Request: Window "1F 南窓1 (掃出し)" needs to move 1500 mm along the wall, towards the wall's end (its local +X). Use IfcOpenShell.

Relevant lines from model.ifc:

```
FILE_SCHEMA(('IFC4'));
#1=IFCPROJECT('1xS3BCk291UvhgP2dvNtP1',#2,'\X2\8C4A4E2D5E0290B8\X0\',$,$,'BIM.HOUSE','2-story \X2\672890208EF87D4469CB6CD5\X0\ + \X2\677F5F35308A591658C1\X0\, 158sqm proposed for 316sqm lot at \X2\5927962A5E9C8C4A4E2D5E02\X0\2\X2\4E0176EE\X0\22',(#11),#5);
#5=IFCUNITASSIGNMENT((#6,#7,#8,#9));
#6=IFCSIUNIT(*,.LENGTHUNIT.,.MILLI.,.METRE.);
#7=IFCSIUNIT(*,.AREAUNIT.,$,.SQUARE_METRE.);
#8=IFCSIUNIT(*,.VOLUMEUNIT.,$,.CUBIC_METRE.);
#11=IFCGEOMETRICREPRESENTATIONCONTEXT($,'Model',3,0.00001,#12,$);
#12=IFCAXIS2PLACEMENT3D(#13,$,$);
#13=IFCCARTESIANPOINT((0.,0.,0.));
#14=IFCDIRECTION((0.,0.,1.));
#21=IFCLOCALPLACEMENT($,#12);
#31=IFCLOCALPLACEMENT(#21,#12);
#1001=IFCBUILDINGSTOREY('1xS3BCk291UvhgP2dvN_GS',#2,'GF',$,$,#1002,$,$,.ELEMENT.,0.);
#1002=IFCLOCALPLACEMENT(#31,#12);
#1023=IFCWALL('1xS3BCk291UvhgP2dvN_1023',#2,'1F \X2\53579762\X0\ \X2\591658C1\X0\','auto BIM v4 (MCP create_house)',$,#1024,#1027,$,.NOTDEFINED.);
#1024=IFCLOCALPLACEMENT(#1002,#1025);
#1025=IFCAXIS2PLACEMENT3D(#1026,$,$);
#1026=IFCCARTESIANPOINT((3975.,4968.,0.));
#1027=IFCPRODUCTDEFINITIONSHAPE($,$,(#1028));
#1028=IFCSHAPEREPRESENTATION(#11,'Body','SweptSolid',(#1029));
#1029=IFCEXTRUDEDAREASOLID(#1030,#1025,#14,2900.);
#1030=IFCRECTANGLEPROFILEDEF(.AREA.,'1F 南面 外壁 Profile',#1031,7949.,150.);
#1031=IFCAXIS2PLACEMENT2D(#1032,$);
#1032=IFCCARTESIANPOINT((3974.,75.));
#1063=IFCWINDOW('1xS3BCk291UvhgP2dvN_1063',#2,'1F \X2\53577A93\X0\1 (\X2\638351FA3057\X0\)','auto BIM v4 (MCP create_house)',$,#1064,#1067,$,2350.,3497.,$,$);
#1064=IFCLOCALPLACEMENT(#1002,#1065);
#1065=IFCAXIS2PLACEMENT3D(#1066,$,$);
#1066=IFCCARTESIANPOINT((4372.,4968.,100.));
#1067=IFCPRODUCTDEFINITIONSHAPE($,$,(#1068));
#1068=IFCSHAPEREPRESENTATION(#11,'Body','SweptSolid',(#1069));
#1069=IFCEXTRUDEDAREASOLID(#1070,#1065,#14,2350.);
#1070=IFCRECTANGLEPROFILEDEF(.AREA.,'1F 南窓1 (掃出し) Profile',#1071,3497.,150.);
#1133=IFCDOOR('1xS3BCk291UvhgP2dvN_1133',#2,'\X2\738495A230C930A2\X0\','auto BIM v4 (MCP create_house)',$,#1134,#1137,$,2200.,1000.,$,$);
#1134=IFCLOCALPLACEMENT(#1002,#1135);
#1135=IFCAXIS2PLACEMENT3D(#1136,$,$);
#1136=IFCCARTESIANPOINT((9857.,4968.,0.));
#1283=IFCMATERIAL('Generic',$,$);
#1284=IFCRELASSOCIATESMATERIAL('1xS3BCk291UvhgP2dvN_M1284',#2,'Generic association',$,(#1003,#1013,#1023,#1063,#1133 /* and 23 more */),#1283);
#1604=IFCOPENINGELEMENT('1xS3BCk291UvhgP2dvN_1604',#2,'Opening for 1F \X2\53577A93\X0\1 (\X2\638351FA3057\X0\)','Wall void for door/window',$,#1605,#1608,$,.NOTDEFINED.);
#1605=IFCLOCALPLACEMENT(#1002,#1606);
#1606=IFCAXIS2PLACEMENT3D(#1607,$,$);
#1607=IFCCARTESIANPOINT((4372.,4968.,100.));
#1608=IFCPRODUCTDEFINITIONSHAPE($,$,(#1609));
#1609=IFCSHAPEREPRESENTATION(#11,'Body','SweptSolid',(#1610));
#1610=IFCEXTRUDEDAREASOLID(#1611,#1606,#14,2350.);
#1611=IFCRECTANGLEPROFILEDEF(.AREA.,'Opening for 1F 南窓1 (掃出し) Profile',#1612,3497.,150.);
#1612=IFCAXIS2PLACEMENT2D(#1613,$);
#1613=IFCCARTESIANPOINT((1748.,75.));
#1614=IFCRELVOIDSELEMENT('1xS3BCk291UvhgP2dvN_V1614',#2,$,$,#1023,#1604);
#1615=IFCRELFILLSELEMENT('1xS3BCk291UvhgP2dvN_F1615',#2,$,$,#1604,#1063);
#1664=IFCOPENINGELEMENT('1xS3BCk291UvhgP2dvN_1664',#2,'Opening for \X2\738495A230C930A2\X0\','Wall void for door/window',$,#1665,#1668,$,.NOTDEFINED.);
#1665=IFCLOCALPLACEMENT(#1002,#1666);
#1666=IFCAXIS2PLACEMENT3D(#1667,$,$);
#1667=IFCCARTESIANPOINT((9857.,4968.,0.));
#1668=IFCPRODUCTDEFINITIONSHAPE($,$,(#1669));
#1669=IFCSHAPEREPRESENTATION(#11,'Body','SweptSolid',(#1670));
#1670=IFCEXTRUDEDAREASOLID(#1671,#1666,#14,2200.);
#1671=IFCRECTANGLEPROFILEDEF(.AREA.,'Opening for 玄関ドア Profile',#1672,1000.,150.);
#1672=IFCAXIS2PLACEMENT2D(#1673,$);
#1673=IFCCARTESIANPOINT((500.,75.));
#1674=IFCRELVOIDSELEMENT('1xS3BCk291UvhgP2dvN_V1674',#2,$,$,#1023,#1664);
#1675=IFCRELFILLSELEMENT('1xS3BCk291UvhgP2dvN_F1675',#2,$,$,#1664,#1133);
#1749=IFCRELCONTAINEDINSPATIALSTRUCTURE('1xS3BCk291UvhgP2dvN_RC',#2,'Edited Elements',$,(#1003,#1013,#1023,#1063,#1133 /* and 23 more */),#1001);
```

```python
import ifcopenshell
import ifcopenshell.api.geometry
import ifcopenshell.util.placement

model = ifcopenshell.open("model.ifc")

window = model.by_id(1063)
opening = window.FillsVoids[0].RelatingOpeningElement
wall = opening.VoidsElements[0].RelatingBuildingElement

wall_matrix = ifcopenshell.util.placement.get_local_placement(wall.ObjectPlacement)
shift = wall_matrix[:3, 0] * 1500.0
before = ifcopenshell.util.placement.get_local_placement(window.ObjectPlacement)[:3, 3].copy()

# The window is not placed relative to its opening, so move both.
for product in (opening, window):
    matrix = ifcopenshell.util.placement.get_local_placement(product.ObjectPlacement)
    matrix[:3, 3] += shift
    ifcopenshell.api.geometry.edit_object_placement(model, product=product, matrix=matrix, is_si=False)

after = ifcopenshell.util.placement.get_local_placement(window.ObjectPlacement)[:3, 3]
print("window moved by", (after - before).round(3) + 0.0)

model.write("model_edited.ifc")
```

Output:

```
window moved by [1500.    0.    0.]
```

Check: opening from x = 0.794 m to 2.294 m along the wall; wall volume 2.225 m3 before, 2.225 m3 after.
